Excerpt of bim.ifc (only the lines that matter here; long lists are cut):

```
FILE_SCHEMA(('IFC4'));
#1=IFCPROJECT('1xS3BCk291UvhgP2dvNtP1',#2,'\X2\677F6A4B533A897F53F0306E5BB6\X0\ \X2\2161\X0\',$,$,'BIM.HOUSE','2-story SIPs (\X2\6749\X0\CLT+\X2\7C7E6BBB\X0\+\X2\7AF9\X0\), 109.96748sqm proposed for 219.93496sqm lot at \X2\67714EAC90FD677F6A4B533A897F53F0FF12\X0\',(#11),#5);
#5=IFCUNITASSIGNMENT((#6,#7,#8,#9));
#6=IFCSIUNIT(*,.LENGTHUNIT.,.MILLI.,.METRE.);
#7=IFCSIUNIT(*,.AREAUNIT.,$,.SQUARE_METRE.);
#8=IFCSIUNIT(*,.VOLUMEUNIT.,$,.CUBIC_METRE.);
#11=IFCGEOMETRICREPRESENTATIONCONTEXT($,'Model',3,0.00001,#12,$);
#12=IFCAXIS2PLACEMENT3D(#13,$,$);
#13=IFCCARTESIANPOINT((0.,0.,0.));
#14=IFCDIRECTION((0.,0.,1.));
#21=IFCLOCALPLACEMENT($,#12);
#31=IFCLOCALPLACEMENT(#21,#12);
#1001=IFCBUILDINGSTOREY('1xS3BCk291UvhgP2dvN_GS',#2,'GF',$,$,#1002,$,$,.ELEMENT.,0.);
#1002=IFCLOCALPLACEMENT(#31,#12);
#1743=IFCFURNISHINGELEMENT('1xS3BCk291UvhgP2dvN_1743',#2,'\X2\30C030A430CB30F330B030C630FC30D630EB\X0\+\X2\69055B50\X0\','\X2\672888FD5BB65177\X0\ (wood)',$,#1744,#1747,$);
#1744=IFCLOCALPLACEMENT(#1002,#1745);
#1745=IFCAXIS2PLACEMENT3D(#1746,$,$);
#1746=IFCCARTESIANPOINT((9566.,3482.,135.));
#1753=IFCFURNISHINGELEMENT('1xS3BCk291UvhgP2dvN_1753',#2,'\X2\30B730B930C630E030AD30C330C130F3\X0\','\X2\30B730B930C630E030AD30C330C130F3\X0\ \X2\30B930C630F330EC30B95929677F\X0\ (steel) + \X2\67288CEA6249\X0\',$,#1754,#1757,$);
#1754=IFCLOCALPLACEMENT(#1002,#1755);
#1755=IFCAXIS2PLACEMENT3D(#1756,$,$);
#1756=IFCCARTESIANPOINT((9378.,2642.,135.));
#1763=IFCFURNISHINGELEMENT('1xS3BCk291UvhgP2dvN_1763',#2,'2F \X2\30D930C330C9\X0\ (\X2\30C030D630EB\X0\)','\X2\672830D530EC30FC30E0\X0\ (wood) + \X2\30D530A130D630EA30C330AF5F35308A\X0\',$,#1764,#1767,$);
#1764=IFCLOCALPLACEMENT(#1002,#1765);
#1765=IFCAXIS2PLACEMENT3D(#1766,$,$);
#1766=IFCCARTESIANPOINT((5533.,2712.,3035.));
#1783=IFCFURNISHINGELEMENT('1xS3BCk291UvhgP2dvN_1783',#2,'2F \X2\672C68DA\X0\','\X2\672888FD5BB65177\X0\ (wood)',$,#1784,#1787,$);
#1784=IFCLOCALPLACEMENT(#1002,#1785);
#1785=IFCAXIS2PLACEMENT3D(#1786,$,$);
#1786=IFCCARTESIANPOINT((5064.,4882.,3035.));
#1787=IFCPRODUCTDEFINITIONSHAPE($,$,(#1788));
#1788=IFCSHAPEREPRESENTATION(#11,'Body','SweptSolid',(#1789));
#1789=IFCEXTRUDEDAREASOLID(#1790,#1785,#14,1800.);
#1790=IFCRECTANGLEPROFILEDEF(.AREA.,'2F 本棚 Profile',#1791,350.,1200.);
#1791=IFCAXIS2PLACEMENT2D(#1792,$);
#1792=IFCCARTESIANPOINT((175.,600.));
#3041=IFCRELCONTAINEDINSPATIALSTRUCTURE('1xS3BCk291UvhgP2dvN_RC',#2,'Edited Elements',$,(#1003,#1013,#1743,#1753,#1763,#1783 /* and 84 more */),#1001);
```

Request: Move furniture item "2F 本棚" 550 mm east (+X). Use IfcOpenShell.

```python
import ifcopenshell
import ifcopenshell.api.geometry
import ifcopenshell.util.placement
import ifcopenshell.util.unit

model = ifcopenshell.open("bim.ifc")
unit_scale = ifcopenshell.util.unit.calculate_unit_scale(model)

item = model.by_guid("1xS3BCk291UvhgP2dvN_1783")
matrix = ifcopenshell.util.placement.get_local_placement(item.ObjectPlacement)
matrix[0, 3] += 0.55 / unit_scale
ifcopenshell.api.geometry.edit_object_placement(model, product=item, matrix=matrix, is_si=False)

print(ifcopenshell.util.placement.get_local_placement(item.ObjectPlacement).round(3) + 0.0)

model.write("bim_v2.ifc")
```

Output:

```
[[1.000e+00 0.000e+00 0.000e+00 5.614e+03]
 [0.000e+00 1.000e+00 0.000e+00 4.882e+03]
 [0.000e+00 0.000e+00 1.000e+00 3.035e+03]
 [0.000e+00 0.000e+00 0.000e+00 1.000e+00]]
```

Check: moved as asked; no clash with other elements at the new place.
